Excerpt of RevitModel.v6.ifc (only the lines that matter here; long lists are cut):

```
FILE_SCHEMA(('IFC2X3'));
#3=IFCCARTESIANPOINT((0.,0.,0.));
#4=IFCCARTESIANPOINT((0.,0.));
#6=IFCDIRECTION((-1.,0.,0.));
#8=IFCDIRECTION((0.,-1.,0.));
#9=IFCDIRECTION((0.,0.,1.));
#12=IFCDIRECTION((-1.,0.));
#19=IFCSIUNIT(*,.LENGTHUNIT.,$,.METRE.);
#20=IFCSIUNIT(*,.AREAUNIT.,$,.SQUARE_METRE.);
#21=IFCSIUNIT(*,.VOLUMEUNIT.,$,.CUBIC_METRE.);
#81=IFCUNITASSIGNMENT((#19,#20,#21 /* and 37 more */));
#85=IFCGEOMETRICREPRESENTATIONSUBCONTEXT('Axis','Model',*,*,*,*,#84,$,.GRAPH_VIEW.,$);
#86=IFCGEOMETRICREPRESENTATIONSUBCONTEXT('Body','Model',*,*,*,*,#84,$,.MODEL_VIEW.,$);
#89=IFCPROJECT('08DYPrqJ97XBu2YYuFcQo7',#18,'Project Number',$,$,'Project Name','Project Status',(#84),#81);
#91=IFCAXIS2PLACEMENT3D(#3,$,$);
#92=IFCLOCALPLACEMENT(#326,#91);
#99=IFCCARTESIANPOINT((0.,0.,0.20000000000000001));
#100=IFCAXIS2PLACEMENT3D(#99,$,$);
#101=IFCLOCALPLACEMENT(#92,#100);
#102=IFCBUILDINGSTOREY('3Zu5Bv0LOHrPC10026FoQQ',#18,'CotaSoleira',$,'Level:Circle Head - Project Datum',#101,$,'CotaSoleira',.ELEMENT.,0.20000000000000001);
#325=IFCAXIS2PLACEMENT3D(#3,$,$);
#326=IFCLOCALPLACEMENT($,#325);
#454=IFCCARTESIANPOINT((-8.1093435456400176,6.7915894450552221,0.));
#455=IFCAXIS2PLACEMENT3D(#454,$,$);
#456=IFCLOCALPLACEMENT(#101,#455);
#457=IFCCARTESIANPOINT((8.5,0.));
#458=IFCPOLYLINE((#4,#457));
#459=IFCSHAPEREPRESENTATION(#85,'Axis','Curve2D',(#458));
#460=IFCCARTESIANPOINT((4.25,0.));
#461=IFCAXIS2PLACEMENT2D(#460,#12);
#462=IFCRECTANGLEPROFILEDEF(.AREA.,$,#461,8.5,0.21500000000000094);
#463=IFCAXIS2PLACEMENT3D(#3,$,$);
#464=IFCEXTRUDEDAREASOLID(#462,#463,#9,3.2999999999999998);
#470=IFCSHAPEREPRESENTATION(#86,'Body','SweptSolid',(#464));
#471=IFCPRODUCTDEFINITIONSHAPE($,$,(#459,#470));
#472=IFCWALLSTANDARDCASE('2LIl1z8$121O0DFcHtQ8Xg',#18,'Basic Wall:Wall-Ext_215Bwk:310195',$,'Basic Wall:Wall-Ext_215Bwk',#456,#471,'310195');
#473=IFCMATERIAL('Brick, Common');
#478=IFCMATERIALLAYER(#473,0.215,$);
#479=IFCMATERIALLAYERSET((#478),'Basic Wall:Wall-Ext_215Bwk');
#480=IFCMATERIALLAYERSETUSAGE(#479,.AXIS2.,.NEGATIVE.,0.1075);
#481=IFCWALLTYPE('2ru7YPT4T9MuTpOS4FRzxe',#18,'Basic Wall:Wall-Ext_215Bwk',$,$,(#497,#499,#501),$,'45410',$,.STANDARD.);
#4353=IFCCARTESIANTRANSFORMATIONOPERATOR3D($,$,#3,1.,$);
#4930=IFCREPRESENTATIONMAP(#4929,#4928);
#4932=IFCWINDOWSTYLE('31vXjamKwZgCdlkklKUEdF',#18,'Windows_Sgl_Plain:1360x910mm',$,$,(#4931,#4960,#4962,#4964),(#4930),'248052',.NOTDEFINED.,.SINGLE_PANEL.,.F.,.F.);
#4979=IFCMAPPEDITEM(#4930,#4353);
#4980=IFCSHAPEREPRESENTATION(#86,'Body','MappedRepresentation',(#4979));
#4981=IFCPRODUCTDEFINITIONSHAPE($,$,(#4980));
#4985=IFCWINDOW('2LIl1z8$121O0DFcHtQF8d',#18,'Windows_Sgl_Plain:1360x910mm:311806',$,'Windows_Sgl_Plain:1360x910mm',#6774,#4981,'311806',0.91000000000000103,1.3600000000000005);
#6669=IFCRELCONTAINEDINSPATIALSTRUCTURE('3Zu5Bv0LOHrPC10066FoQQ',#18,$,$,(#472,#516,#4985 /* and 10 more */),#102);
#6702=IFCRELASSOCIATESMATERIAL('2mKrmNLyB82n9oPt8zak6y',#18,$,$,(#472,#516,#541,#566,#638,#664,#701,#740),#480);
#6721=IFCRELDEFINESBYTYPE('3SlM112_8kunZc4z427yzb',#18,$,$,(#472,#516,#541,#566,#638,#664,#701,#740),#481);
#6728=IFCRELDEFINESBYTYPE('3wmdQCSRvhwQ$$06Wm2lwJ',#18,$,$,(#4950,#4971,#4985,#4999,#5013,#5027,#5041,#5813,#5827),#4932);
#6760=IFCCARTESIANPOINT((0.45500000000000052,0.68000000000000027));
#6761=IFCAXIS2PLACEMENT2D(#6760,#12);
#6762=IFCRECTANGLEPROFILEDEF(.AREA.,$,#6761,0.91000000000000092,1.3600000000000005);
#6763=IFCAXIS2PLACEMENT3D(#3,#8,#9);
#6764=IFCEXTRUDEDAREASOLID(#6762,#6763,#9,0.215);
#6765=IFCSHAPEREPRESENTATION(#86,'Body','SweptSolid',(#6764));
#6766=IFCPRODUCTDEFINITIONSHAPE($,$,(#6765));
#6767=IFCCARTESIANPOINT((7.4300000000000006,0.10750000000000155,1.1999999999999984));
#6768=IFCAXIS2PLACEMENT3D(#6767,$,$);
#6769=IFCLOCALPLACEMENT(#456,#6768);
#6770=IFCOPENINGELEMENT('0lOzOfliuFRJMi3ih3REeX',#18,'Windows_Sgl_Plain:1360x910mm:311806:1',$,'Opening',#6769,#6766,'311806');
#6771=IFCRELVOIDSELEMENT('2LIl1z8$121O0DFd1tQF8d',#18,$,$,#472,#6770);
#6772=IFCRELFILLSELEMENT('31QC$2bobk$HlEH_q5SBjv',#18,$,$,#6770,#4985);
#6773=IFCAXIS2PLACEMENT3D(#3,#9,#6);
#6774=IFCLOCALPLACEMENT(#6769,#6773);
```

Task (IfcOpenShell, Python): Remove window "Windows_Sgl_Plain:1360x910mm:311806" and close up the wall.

```python
import ifcopenshell
import ifcopenshell.api.feature
import ifcopenshell.api.root
import ifcopenshell.geom
import ifcopenshell.util.shape

model = ifcopenshell.open("RevitModel.v6.ifc")
settings = ifcopenshell.geom.settings()


def volume(element):
    """Net volume in cubic metres, openings subtracted."""
    shape = ifcopenshell.geom.create_shape(settings, element)
    return ifcopenshell.util.shape.get_volume(shape.geometry)


window = model.by_guid("2LIl1z8$121O0DFcHtQF8d")
opening = window.FillsVoids[0].RelatingOpeningElement
wall = opening.VoidsElements[0].RelatingBuildingElement
before = volume(wall)

ifcopenshell.api.root.remove_product(model, product=window)
ifcopenshell.api.feature.remove_feature(model, feature=opening)

after = volume(wall)

print(f"wall volume {before:.3f} -> {after:.3f} m3")

model.write("RevitModel.v6_rev.ifc")
```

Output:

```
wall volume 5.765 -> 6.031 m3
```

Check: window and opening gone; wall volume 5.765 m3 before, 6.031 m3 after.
